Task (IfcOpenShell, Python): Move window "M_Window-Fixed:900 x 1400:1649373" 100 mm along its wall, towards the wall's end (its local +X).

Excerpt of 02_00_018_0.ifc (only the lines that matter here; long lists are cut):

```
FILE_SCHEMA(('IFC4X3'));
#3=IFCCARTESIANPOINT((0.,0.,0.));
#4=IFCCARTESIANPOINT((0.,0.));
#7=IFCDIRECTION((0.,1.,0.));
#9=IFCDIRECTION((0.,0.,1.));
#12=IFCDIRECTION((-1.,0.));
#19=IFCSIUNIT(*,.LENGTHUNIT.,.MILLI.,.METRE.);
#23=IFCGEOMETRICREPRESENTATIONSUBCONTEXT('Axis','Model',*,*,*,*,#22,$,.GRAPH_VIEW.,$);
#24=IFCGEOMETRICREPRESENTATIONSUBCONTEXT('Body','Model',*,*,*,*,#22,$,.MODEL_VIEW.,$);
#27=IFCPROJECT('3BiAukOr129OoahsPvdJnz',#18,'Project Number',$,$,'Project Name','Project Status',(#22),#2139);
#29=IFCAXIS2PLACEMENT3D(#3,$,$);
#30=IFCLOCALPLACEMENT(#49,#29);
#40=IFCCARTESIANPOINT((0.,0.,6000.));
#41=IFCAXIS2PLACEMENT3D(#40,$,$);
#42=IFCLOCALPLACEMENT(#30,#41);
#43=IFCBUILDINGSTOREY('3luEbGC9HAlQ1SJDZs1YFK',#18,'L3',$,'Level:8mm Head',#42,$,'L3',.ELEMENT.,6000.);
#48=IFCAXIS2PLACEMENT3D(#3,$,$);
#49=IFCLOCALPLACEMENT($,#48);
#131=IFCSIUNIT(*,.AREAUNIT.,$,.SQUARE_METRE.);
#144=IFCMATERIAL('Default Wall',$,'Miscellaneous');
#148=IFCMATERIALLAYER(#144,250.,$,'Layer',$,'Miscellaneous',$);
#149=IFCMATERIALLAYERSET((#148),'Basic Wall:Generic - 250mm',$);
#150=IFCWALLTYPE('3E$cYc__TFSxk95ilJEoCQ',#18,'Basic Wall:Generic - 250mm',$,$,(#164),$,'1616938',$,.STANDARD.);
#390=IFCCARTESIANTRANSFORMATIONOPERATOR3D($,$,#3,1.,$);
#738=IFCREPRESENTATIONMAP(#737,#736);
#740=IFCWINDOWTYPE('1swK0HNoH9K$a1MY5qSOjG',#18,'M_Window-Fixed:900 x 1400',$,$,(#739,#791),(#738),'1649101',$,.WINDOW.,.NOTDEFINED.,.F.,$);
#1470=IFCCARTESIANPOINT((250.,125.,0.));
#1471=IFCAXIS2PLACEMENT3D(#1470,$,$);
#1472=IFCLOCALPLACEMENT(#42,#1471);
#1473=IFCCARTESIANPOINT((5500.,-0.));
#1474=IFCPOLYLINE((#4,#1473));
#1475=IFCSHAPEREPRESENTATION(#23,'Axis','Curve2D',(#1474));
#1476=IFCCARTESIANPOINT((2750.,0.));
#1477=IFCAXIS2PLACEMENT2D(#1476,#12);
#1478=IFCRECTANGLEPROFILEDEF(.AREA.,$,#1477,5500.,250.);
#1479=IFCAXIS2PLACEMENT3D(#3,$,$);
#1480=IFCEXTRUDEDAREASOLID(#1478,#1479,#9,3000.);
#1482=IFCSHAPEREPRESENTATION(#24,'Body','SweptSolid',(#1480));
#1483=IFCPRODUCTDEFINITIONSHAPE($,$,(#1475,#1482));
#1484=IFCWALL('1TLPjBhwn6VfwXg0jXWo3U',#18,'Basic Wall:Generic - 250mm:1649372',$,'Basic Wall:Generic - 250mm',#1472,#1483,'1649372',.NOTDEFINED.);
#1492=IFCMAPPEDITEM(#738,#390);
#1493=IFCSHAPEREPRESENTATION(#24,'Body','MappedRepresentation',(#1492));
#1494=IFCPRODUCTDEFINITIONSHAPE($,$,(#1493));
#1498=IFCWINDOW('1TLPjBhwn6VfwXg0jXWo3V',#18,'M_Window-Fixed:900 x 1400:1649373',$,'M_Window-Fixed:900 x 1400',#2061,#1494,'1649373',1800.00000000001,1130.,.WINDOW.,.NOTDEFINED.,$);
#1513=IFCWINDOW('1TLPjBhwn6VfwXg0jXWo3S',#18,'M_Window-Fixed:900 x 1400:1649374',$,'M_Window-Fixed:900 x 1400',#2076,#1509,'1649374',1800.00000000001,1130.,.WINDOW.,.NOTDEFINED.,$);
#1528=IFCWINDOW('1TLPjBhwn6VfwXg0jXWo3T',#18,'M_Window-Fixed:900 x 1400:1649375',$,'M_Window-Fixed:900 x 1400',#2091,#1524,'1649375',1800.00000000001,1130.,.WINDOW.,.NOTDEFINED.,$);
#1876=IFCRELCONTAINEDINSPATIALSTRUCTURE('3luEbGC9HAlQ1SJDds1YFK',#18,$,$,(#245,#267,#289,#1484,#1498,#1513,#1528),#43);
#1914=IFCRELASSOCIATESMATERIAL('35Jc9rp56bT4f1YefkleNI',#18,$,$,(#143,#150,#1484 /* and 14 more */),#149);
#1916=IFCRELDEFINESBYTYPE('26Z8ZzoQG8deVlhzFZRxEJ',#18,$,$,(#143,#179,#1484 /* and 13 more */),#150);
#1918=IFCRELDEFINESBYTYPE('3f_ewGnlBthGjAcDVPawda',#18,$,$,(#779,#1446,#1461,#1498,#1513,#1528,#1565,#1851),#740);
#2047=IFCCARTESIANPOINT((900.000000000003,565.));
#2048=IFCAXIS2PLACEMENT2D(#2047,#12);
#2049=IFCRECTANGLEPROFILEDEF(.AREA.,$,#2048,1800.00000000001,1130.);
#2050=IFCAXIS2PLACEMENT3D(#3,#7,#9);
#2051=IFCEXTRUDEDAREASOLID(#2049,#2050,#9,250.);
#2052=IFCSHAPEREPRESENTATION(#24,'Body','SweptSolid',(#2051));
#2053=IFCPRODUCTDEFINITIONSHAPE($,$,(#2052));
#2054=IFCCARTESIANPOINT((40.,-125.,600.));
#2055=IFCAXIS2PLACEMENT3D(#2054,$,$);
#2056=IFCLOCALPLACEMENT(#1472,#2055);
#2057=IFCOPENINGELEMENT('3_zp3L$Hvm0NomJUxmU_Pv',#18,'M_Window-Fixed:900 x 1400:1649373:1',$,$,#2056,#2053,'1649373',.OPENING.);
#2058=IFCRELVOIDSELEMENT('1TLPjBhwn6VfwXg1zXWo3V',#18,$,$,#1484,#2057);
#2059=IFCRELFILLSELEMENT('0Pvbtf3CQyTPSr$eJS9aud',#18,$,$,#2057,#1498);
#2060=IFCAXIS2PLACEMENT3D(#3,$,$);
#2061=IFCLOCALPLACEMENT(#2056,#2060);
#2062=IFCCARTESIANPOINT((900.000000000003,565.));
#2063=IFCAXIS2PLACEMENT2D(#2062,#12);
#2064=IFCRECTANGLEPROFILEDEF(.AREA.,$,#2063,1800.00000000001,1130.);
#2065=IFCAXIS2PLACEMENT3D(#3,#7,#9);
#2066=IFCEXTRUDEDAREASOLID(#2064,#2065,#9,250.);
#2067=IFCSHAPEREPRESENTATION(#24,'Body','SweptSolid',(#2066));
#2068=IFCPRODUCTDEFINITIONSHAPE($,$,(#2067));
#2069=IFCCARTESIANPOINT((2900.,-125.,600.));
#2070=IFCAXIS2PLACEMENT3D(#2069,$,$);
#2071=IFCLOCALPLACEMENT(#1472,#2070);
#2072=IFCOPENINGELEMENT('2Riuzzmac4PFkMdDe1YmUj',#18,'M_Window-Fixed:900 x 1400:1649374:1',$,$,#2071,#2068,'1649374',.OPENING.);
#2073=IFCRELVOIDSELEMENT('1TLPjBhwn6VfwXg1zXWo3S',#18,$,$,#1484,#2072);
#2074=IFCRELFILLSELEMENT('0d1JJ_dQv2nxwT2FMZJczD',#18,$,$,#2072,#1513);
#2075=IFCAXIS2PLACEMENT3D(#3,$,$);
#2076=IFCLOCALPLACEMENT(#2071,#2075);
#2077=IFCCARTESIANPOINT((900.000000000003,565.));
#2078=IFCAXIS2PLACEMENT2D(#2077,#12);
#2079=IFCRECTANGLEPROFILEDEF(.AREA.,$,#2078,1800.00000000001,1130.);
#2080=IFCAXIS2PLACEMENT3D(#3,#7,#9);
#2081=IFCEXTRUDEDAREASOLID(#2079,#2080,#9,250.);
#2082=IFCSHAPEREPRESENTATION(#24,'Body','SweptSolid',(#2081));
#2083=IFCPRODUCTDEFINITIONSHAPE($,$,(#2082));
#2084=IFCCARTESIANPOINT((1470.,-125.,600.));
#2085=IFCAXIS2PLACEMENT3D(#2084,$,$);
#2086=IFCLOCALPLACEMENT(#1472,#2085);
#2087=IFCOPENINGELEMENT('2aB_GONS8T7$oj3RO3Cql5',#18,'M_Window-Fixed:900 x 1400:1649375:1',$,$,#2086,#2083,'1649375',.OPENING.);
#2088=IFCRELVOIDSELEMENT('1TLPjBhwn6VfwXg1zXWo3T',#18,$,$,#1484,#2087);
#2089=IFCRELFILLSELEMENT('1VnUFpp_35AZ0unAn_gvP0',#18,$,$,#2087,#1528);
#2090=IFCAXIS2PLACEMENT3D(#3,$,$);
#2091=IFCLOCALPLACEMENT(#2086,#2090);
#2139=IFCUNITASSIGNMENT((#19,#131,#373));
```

```python
import ifcopenshell
import ifcopenshell.api.geometry
import ifcopenshell.util.placement
import ifcopenshell.util.unit

model = ifcopenshell.open("02_00_018_0.ifc")
unit_scale = ifcopenshell.util.unit.calculate_unit_scale(model)

window = model.by_guid("1TLPjBhwn6VfwXg0jXWo3V")
opening = window.FillsVoids[0].RelatingOpeningElement
wall = opening.VoidsElements[0].RelatingBuildingElement

wall_matrix = ifcopenshell.util.placement.get_local_placement(wall.ObjectPlacement)
shift = wall_matrix[:3, 0] * 0.1 / unit_scale
before = ifcopenshell.util.placement.get_local_placement(window.ObjectPlacement)[:3, 3].copy()

# The window is placed relative to its opening, so it follows when the opening moves.
matrix = ifcopenshell.util.placement.get_local_placement(opening.ObjectPlacement)
matrix[:3, 3] += shift
ifcopenshell.api.geometry.edit_object_placement(
    model, product=opening, matrix=matrix, is_si=False, should_transform_children=True
)

after = ifcopenshell.util.placement.get_local_placement(window.ObjectPlacement)[:3, 3]
print("window moved by", (after - before).round(3) + 0.0)

model.write("02_00_018_0_v2.ifc")
```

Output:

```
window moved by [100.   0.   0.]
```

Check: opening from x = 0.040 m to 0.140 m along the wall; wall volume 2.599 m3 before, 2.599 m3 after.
